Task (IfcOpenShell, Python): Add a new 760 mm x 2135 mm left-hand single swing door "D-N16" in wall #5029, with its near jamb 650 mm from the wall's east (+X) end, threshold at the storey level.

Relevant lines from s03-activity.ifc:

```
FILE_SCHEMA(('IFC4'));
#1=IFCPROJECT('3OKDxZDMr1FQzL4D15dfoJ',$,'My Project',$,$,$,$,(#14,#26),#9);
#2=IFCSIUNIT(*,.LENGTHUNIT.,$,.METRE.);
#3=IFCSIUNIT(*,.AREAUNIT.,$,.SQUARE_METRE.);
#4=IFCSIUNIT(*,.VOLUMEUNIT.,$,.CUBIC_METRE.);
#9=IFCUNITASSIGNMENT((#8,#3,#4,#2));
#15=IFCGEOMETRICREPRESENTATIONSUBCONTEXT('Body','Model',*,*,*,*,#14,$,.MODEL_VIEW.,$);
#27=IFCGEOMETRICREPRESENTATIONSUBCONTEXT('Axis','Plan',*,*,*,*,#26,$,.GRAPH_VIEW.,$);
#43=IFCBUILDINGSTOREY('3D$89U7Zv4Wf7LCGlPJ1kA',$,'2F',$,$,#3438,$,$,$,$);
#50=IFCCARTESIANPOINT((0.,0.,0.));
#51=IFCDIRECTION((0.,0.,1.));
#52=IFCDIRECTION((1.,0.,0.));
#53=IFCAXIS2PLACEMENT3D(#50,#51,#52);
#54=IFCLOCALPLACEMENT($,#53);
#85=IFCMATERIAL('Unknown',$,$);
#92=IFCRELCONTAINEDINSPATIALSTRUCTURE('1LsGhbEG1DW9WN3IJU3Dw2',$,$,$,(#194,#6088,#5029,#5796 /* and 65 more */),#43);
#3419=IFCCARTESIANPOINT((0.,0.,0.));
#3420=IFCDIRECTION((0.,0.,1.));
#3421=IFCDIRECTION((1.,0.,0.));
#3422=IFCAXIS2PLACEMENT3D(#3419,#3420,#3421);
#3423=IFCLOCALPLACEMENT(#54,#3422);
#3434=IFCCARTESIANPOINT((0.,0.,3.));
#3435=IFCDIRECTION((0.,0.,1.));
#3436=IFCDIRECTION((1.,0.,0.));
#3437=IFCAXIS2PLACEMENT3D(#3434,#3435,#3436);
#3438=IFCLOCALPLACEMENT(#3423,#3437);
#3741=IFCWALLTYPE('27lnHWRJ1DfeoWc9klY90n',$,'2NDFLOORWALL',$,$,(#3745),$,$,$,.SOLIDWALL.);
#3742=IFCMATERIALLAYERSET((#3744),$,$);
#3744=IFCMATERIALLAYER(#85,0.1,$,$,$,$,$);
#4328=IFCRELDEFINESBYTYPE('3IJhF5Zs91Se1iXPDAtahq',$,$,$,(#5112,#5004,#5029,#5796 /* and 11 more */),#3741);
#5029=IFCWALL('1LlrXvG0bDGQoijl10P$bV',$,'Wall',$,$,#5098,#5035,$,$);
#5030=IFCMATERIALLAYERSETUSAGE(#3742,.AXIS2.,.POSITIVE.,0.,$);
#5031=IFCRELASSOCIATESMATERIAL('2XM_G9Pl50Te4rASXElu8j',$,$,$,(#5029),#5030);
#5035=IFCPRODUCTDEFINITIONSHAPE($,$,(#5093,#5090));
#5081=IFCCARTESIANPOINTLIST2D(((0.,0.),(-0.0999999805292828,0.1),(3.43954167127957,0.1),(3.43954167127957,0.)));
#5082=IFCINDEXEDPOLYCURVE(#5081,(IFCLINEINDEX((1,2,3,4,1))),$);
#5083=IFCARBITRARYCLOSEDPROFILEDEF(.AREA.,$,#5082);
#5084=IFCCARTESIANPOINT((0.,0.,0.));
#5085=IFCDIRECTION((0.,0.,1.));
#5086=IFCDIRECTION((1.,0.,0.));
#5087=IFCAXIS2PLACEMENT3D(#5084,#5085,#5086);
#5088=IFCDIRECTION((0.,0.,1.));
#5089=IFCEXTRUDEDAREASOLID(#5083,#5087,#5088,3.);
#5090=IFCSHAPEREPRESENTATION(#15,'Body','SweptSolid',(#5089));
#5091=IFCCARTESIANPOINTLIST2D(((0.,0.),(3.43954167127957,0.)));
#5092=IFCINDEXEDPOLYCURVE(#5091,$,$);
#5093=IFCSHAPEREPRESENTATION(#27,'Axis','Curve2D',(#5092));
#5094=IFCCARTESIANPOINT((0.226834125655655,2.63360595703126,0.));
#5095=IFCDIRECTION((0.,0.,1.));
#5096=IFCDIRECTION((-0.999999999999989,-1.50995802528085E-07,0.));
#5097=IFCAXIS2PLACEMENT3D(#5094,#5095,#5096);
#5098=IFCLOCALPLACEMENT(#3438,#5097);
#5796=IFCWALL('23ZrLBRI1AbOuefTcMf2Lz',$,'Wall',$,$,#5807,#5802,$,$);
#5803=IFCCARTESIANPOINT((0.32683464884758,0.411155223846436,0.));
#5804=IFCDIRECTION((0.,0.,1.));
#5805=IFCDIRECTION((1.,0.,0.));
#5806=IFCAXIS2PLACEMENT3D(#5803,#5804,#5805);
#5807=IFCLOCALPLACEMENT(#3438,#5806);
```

```python
import numpy as np
import ifcopenshell
import ifcopenshell.api.feature
import ifcopenshell.api.geometry
import ifcopenshell.api.root
import ifcopenshell.api.spatial
import ifcopenshell.geom
import ifcopenshell.util.element
import ifcopenshell.util.placement
import ifcopenshell.util.representation
import ifcopenshell.util.shape
import ifcopenshell.util.unit

model = ifcopenshell.open("s03-activity.ifc")
unit_scale = ifcopenshell.util.unit.calculate_unit_scale(model)
settings = ifcopenshell.geom.settings()


def volume(element):
    """Net volume in cubic metres, openings subtracted."""
    shape = ifcopenshell.geom.create_shape(settings, element)
    return ifcopenshell.util.shape.get_volume(shape.geometry)


wall = model.by_id(5029)
storey = ifcopenshell.util.element.get_container(wall, ifc_class="IfcBuildingStorey")
context = ifcopenshell.util.representation.get_context(model, "Model", "Body", "MODEL_VIEW")
before = volume(wall)

width, height, from_end, sill = 0.76, 2.135, 0.65, 0.0  # metres

# The wall runs along its own X axis, and the end named is its -X end.
wall_shape = ifcopenshell.geom.create_shape(settings, wall)
x, y, z = ifcopenshell.util.shape.get_vertices(wall_shape.geometry).T
start = x.min() + from_end
face, thickness = float(y.min()), float(y.max() - y.min())
wall_matrix = ifcopenshell.util.placement.get_local_placement(wall.ObjectPlacement)
level = ifcopenshell.util.placement.get_local_placement(storey.ObjectPlacement)[2, 3]


def in_wall(x, y):
    """Placement at x, y metres in the wall's axes, at sill height."""
    matrix = wall_matrix.copy()
    matrix[:, 3] = wall_matrix @ np.array([x / unit_scale, y / unit_scale, 0.0, 1.0])
    matrix[2, 3] = level + sill / unit_scale
    return matrix


# Opening: a box that overshoots both wall faces by 50 mm.
opening = ifcopenshell.api.root.create_entity(model, ifc_class="IfcOpeningElement", predefined_type="OPENING")
box = ifcopenshell.api.geometry.add_wall_representation(
    model, context=context, length=width, height=height, thickness=thickness + 0.1
)
ifcopenshell.api.geometry.assign_representation(model, product=opening, representation=box)
ifcopenshell.api.geometry.edit_object_placement(model, product=opening, matrix=in_wall(start, face - 0.05), is_si=False)
ifcopenshell.api.feature.add_feature(model, feature=opening, element=wall)

door = ifcopenshell.api.root.create_entity(model, ifc_class="IfcDoor", name="D-N16", predefined_type="DOOR")
door.OverallWidth, door.OverallHeight = width / unit_scale, height / unit_scale
door.OperationType = "SINGLE_SWING_LEFT"
body = ifcopenshell.api.geometry.add_door_representation(
    model,
    context=context,
    overall_width=door.OverallWidth,
    overall_height=door.OverallHeight,
    operation_type="SINGLE_SWING_LEFT",
    lining_properties={"LiningDepth": thickness / unit_scale, "ThresholdDepth": thickness / unit_scale},
)
ifcopenshell.api.geometry.assign_representation(model, product=door, representation=body)
ifcopenshell.api.spatial.assign_container(model, products=[door], relating_structure=storey)
ifcopenshell.api.feature.add_filling(model, opening=opening, element=door)

# The lining spans the wall, so the door starts at the wall face.
ifcopenshell.api.geometry.edit_object_placement(model, product=door, matrix=in_wall(start, face), is_si=False)

after = volume(wall)

print(f"wall volume {before:.3f} -> {after:.3f} m3")

model.write("s03-activity-out.ifc")
```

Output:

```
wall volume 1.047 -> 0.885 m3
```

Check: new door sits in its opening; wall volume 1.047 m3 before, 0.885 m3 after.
